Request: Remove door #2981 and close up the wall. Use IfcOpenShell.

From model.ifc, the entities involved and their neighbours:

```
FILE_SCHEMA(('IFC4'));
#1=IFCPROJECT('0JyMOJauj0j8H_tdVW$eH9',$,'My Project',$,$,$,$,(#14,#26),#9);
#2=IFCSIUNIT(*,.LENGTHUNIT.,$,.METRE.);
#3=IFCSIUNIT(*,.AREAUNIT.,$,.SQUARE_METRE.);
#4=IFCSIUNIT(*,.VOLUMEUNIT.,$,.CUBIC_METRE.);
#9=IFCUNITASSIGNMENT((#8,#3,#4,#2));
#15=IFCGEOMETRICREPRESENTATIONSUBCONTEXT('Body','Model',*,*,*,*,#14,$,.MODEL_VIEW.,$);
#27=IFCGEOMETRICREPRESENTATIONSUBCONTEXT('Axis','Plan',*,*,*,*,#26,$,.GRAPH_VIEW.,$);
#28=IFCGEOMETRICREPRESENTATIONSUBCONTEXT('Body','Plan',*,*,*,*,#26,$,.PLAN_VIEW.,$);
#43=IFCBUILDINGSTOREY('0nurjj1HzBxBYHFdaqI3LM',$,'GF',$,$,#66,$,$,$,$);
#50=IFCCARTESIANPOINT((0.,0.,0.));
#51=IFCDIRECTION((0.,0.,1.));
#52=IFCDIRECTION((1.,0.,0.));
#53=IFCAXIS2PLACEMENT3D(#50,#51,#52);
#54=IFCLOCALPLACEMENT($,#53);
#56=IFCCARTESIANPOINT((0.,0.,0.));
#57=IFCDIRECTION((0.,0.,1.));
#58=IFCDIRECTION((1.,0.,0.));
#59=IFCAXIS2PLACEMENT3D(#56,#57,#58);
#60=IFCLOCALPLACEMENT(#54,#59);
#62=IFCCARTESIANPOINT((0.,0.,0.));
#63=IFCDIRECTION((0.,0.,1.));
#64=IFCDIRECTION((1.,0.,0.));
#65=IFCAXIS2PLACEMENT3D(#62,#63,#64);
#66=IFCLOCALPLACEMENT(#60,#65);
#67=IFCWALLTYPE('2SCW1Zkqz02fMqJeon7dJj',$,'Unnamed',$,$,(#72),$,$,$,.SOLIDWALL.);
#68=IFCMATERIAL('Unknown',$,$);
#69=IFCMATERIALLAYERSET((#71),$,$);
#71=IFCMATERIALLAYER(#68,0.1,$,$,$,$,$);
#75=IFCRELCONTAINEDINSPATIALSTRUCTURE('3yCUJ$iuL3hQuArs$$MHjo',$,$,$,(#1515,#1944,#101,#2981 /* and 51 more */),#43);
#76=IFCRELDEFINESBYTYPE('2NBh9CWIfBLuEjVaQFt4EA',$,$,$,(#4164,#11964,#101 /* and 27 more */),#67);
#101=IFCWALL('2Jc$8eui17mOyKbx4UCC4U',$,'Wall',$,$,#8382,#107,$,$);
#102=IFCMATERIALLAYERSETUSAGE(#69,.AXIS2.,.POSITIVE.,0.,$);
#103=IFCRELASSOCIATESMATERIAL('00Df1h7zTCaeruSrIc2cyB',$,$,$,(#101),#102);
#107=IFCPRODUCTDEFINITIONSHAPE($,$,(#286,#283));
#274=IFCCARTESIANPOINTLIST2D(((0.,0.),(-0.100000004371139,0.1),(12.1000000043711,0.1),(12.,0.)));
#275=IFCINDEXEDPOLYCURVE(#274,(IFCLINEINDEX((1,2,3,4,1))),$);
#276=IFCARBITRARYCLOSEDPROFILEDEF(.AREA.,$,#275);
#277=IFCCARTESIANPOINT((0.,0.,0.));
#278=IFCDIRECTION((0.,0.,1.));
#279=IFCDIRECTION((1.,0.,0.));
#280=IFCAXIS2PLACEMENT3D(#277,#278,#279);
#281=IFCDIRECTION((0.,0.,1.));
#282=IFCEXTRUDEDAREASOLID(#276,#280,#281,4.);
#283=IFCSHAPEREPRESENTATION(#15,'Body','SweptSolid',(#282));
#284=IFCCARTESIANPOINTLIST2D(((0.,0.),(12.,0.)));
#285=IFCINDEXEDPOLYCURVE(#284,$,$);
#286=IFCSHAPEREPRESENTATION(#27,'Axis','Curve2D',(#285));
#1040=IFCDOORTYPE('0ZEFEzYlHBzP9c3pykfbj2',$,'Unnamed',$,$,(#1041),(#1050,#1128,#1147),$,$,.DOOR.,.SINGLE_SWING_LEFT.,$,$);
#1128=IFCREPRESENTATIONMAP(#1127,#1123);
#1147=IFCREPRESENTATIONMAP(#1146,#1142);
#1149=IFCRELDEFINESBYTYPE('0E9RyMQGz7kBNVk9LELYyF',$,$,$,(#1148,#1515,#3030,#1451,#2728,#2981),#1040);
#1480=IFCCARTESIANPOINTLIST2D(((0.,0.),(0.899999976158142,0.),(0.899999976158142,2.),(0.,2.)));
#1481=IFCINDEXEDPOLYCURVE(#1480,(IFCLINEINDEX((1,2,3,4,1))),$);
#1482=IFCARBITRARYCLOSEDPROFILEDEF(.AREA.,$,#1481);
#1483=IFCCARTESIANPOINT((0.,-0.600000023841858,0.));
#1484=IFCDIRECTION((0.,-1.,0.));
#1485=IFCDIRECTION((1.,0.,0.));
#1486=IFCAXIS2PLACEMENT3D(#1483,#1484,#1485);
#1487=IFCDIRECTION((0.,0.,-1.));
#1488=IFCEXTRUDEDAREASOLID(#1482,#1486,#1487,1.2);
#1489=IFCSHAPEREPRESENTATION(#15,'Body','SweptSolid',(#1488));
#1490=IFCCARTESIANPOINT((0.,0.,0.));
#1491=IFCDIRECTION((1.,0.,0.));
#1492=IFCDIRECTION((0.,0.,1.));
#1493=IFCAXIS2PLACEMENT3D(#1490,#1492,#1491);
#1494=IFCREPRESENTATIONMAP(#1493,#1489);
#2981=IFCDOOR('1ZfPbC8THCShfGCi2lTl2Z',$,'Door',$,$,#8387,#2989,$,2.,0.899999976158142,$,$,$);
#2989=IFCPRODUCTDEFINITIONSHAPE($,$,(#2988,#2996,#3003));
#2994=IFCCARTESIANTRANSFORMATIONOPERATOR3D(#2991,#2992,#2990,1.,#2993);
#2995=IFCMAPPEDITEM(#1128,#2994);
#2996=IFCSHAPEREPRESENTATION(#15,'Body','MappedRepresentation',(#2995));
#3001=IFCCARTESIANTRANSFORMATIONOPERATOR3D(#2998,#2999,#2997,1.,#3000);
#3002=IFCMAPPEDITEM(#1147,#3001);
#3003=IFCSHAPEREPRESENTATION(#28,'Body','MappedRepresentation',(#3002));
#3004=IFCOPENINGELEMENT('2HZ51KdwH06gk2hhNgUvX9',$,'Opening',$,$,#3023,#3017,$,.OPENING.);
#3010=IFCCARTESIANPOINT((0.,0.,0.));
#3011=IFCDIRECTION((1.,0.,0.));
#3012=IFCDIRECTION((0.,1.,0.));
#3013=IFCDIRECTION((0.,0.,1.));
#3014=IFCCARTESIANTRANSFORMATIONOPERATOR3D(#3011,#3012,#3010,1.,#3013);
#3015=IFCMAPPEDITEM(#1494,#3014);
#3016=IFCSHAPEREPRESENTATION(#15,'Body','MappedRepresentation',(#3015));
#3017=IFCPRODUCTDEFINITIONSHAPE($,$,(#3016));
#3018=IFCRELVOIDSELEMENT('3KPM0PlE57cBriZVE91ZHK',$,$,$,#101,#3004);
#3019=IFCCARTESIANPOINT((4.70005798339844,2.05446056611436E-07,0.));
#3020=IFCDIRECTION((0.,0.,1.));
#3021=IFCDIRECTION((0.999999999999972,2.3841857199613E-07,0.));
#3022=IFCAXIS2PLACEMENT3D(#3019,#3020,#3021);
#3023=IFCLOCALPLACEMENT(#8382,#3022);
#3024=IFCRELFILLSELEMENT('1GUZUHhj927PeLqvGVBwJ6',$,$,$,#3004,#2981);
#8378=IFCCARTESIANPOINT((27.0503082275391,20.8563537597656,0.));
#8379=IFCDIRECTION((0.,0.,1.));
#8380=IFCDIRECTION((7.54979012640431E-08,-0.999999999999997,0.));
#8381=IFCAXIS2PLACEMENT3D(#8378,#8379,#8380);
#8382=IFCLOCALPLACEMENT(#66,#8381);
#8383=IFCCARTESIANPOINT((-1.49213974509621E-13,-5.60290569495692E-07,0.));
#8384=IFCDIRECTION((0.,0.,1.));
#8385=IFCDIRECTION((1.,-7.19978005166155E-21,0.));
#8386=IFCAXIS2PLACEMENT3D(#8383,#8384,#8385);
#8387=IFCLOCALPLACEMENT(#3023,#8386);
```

```python
import ifcopenshell
import ifcopenshell.api.feature
import ifcopenshell.api.root
import ifcopenshell.geom
import ifcopenshell.util.shape

model = ifcopenshell.open("model.ifc")
settings = ifcopenshell.geom.settings()


def volume(element):
    """Net volume in cubic metres, openings subtracted."""
    shape = ifcopenshell.geom.create_shape(settings, element)
    return ifcopenshell.util.shape.get_volume(shape.geometry)


door = model.by_guid("1ZfPbC8THCShfGCi2lTl2Z")
opening = door.FillsVoids[0].RelatingOpeningElement
wall = opening.VoidsElements[0].RelatingBuildingElement
before = volume(wall)

ifcopenshell.api.root.remove_product(model, product=door)
ifcopenshell.api.feature.remove_feature(model, feature=opening)

after = volume(wall)

print(f"wall volume {before:.3f} -> {after:.3f} m3")

model.write("model_edited.ifc")
```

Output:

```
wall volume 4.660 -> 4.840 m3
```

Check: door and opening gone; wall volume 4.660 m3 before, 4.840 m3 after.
